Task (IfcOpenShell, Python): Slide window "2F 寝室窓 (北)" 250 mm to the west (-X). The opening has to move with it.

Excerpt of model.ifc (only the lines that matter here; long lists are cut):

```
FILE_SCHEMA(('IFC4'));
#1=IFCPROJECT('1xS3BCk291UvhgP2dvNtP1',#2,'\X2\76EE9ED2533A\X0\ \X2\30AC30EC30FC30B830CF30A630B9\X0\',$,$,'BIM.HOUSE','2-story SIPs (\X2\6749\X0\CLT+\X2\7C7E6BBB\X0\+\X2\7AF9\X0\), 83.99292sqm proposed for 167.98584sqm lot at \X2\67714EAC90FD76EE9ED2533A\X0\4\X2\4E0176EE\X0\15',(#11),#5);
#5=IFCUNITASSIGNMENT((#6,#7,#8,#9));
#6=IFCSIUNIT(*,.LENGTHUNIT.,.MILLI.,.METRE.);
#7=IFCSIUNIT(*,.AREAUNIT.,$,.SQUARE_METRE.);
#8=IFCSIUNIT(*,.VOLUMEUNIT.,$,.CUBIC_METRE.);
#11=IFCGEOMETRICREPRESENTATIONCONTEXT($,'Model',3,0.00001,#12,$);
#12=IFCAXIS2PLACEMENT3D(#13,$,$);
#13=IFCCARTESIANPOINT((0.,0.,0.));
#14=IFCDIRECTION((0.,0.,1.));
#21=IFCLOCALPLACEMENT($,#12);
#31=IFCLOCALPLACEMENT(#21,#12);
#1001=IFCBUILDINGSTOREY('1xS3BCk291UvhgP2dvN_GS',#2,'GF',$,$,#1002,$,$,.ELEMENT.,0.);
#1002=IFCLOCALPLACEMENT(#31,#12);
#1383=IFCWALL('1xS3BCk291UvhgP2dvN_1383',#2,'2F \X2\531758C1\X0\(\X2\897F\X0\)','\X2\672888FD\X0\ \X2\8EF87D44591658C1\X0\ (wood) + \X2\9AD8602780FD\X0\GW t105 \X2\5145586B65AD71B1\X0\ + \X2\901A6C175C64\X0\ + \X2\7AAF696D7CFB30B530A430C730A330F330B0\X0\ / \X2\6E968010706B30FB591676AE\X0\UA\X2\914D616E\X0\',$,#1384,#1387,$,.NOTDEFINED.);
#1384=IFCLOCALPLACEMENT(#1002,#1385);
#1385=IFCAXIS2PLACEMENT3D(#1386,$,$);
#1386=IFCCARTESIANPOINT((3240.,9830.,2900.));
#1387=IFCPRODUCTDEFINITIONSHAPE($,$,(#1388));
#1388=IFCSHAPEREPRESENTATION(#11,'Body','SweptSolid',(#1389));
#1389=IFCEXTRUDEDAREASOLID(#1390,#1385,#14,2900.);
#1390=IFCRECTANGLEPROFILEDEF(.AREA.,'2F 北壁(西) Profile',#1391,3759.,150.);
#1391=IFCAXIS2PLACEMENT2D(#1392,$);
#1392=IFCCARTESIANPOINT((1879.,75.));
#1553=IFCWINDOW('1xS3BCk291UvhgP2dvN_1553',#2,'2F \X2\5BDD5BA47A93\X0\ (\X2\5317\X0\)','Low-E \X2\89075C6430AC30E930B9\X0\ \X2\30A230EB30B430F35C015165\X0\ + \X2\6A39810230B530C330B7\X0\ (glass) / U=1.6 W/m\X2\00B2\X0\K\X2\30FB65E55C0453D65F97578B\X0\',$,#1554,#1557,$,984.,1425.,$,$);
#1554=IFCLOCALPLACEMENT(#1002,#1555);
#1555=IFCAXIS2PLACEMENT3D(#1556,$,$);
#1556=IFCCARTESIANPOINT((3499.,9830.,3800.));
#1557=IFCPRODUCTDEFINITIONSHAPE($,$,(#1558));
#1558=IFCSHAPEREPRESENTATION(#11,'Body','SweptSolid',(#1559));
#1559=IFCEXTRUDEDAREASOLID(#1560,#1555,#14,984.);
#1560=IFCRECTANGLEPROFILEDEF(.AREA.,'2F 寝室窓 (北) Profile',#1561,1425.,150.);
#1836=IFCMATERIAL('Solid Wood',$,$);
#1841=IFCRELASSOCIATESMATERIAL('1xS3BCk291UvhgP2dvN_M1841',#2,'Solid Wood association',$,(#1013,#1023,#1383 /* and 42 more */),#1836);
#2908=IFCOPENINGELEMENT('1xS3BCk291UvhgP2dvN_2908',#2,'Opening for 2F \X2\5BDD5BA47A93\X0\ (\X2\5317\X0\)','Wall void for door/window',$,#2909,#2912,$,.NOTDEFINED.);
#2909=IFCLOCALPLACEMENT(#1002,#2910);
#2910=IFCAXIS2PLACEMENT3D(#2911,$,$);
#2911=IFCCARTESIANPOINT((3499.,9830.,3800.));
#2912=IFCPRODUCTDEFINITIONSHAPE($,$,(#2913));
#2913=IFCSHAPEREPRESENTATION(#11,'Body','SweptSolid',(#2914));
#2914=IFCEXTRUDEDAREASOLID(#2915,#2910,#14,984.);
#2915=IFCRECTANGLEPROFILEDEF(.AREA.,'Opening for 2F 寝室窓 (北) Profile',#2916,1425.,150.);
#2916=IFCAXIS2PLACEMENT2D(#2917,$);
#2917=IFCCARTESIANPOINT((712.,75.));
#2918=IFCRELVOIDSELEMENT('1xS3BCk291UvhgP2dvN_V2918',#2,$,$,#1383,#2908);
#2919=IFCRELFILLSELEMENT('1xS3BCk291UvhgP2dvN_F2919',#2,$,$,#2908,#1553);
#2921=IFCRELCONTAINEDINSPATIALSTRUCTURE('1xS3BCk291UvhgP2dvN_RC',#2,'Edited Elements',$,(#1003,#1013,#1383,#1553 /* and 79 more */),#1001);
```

```python
import ifcopenshell
import ifcopenshell.api.geometry
import ifcopenshell.util.placement

model = ifcopenshell.open("model.ifc")

window = model.by_id(1553)
opening = window.FillsVoids[0].RelatingOpeningElement
wall = opening.VoidsElements[0].RelatingBuildingElement

wall_matrix = ifcopenshell.util.placement.get_local_placement(wall.ObjectPlacement)
shift = wall_matrix[:3, 0] * -250.0
before = ifcopenshell.util.placement.get_local_placement(window.ObjectPlacement)[:3, 3].copy()

# The window is not placed relative to its opening, so move both.
for product in (opening, window):
    matrix = ifcopenshell.util.placement.get_local_placement(product.ObjectPlacement)
    matrix[:3, 3] += shift
    ifcopenshell.api.geometry.edit_object_placement(model, product=product, matrix=matrix, is_si=False)

after = ifcopenshell.util.placement.get_local_placement(window.ObjectPlacement)[:3, 3]
print("window moved by", (after - before).round(3) + 0.0)

model.write("model_edited.ifc")
```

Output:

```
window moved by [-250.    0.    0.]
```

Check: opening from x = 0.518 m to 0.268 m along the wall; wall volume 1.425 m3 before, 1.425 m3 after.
